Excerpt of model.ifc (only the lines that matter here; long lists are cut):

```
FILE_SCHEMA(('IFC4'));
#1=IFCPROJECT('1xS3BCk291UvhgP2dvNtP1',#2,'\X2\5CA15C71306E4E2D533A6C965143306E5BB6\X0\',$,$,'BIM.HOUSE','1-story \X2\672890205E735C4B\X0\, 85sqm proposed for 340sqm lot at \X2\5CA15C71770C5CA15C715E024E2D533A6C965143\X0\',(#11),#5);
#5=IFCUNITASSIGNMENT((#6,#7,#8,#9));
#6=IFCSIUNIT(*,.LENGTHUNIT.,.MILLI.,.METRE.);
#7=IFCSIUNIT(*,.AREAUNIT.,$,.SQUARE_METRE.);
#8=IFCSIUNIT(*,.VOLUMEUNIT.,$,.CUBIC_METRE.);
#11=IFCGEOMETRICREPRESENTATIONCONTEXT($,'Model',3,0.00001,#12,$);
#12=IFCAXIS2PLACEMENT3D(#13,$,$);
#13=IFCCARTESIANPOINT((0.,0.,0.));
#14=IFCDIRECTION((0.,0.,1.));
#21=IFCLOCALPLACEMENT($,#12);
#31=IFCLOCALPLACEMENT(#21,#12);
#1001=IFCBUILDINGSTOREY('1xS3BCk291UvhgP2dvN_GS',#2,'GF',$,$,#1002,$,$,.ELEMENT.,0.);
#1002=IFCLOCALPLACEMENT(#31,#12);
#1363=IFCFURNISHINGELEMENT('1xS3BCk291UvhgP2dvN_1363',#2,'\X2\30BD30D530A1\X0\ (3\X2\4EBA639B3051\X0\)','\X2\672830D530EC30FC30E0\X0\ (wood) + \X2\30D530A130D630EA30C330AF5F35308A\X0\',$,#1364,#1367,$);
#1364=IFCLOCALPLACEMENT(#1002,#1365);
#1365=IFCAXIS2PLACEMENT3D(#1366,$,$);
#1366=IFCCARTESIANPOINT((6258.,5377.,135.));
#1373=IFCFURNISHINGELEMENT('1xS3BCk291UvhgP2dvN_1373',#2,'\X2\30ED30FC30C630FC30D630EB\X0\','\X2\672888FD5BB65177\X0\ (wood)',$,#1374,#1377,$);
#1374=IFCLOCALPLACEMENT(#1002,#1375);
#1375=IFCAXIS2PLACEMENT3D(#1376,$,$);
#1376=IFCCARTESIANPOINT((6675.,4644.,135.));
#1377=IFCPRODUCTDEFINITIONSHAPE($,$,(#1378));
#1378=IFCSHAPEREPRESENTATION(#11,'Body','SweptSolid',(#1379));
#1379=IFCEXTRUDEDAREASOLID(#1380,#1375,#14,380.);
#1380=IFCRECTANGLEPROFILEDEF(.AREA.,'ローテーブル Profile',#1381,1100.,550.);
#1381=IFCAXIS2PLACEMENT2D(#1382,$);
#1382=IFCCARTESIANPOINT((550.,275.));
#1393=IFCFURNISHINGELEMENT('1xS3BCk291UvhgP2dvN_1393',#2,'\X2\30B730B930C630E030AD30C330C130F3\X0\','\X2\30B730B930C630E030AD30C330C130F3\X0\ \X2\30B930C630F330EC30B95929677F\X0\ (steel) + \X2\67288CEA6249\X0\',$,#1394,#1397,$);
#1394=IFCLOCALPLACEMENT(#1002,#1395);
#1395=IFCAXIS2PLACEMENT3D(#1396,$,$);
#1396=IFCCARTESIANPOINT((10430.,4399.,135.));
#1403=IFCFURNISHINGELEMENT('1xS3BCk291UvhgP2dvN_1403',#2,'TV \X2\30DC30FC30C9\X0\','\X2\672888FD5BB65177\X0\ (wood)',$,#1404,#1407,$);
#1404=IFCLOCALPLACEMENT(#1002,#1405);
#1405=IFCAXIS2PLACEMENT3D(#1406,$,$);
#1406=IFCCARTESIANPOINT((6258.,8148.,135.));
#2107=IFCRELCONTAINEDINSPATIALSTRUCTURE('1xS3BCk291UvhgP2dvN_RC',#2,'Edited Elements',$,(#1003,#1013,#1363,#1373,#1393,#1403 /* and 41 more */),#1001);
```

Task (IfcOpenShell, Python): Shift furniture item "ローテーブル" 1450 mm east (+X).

```python
import ifcopenshell
import ifcopenshell.api.geometry
import ifcopenshell.util.placement

model = ifcopenshell.open("model.ifc")

item = model.by_guid("1xS3BCk291UvhgP2dvN_1373")
matrix = ifcopenshell.util.placement.get_local_placement(item.ObjectPlacement)
matrix[0, 3] += 1450.0
ifcopenshell.api.geometry.edit_object_placement(model, product=item, matrix=matrix, is_si=False)

print(ifcopenshell.util.placement.get_local_placement(item.ObjectPlacement).round(3) + 0.0)

model.write("model_rev.ifc")
```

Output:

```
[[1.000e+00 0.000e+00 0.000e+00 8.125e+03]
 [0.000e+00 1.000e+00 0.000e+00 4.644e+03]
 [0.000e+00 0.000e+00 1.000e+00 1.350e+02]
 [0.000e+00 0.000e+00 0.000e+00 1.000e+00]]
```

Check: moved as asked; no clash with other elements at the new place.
